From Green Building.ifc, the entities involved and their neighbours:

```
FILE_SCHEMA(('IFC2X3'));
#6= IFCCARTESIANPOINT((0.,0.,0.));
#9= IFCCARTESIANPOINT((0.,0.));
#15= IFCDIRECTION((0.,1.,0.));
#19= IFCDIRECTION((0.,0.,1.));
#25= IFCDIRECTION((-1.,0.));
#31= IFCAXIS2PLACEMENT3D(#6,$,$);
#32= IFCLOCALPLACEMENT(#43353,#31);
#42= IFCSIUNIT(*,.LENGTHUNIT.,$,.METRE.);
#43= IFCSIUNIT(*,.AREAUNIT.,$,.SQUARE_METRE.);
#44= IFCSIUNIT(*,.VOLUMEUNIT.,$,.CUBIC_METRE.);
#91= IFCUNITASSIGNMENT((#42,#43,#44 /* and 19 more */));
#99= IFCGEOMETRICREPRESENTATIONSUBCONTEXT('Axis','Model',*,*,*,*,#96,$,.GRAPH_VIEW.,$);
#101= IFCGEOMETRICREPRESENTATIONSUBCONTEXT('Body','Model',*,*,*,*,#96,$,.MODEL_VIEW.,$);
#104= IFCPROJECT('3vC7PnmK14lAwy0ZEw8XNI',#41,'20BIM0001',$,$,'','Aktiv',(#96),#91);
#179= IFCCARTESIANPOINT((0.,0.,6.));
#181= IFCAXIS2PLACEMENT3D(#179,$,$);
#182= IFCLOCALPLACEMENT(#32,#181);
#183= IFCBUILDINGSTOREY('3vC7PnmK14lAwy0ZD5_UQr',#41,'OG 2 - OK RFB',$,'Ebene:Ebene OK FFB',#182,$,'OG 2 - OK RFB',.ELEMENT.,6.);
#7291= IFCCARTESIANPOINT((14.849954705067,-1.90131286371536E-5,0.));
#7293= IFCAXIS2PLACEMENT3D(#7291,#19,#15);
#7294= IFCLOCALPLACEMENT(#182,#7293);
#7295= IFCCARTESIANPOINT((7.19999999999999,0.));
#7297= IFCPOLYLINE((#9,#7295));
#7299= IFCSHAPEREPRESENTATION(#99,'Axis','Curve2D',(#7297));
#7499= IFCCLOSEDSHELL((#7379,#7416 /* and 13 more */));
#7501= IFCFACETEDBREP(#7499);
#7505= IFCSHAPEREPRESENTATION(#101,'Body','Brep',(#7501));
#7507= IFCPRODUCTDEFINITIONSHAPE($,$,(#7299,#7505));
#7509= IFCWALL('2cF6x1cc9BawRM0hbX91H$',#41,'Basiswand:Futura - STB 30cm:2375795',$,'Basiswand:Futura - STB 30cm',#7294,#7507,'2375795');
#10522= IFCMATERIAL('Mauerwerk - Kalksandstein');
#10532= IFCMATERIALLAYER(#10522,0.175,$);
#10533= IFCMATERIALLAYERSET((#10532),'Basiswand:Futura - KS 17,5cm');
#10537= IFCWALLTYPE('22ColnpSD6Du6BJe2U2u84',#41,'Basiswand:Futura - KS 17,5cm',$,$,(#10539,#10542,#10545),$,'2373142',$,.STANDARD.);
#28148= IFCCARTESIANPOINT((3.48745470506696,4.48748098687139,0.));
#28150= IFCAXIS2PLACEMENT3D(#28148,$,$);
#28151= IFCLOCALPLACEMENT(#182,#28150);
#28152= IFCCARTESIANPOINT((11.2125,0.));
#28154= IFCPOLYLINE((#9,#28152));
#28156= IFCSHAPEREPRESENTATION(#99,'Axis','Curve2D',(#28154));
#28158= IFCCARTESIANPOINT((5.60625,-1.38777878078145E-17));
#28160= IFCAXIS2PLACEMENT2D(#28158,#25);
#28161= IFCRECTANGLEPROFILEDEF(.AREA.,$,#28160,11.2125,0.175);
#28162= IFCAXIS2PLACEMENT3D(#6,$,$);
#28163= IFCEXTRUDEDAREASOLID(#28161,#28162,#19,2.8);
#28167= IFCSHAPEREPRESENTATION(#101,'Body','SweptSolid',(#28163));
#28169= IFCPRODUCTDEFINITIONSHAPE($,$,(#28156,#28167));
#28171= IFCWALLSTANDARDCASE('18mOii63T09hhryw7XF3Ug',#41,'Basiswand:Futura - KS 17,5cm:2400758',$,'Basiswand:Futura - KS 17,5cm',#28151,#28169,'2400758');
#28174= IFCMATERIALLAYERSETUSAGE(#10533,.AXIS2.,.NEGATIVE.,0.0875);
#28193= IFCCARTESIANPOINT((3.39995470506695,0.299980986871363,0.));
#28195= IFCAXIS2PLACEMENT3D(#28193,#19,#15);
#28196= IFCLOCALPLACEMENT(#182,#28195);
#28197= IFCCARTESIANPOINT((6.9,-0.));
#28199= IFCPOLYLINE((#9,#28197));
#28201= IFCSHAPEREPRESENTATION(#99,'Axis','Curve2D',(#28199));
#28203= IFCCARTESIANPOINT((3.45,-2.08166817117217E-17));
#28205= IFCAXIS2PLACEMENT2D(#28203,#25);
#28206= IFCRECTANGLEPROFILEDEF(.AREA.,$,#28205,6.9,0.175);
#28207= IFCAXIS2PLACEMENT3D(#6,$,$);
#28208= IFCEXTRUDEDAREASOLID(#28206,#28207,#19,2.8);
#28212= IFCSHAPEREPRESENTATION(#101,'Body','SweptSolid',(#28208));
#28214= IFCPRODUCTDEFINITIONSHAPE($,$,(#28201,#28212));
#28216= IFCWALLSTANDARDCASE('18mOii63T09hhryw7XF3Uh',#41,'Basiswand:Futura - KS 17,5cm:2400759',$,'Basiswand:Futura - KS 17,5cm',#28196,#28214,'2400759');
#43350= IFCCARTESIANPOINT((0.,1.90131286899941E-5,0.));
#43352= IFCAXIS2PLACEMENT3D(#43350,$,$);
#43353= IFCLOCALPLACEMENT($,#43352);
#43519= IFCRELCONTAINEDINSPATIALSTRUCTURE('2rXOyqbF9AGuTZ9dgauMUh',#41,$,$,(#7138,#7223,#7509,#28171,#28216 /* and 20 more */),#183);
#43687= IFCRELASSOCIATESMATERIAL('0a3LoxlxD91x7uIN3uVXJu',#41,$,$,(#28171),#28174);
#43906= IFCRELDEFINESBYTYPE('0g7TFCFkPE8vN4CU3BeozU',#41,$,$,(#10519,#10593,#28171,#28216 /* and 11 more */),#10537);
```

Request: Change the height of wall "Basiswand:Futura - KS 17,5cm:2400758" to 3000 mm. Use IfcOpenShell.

```python
import ifcopenshell
import ifcopenshell.geom
import ifcopenshell.util.representation
import ifcopenshell.util.shape
import ifcopenshell.util.unit

model = ifcopenshell.open("Green Building.ifc")
unit_scale = ifcopenshell.util.unit.calculate_unit_scale(model)
settings = ifcopenshell.geom.settings()


def volume(element):
    """Net volume in cubic metres, openings subtracted."""
    shape = ifcopenshell.geom.create_shape(settings, element)
    return ifcopenshell.util.shape.get_volume(shape.geometry)


wall = model.by_guid("18mOii63T09hhryw7XF3Ug")
before = volume(wall)

body = ifcopenshell.util.representation.get_representation(wall, "Model", "Body")
solid = body.Items[0]
old_height = solid.Depth
solid.Depth = 3 / unit_scale
after = volume(wall)

print(f"height {old_height:g} -> {solid.Depth:g}, volume {before:.3f} -> {after:.3f} m3")

model.write("Green Building_edited.ifc")
```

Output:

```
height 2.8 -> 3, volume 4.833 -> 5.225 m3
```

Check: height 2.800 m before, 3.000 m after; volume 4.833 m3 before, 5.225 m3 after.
